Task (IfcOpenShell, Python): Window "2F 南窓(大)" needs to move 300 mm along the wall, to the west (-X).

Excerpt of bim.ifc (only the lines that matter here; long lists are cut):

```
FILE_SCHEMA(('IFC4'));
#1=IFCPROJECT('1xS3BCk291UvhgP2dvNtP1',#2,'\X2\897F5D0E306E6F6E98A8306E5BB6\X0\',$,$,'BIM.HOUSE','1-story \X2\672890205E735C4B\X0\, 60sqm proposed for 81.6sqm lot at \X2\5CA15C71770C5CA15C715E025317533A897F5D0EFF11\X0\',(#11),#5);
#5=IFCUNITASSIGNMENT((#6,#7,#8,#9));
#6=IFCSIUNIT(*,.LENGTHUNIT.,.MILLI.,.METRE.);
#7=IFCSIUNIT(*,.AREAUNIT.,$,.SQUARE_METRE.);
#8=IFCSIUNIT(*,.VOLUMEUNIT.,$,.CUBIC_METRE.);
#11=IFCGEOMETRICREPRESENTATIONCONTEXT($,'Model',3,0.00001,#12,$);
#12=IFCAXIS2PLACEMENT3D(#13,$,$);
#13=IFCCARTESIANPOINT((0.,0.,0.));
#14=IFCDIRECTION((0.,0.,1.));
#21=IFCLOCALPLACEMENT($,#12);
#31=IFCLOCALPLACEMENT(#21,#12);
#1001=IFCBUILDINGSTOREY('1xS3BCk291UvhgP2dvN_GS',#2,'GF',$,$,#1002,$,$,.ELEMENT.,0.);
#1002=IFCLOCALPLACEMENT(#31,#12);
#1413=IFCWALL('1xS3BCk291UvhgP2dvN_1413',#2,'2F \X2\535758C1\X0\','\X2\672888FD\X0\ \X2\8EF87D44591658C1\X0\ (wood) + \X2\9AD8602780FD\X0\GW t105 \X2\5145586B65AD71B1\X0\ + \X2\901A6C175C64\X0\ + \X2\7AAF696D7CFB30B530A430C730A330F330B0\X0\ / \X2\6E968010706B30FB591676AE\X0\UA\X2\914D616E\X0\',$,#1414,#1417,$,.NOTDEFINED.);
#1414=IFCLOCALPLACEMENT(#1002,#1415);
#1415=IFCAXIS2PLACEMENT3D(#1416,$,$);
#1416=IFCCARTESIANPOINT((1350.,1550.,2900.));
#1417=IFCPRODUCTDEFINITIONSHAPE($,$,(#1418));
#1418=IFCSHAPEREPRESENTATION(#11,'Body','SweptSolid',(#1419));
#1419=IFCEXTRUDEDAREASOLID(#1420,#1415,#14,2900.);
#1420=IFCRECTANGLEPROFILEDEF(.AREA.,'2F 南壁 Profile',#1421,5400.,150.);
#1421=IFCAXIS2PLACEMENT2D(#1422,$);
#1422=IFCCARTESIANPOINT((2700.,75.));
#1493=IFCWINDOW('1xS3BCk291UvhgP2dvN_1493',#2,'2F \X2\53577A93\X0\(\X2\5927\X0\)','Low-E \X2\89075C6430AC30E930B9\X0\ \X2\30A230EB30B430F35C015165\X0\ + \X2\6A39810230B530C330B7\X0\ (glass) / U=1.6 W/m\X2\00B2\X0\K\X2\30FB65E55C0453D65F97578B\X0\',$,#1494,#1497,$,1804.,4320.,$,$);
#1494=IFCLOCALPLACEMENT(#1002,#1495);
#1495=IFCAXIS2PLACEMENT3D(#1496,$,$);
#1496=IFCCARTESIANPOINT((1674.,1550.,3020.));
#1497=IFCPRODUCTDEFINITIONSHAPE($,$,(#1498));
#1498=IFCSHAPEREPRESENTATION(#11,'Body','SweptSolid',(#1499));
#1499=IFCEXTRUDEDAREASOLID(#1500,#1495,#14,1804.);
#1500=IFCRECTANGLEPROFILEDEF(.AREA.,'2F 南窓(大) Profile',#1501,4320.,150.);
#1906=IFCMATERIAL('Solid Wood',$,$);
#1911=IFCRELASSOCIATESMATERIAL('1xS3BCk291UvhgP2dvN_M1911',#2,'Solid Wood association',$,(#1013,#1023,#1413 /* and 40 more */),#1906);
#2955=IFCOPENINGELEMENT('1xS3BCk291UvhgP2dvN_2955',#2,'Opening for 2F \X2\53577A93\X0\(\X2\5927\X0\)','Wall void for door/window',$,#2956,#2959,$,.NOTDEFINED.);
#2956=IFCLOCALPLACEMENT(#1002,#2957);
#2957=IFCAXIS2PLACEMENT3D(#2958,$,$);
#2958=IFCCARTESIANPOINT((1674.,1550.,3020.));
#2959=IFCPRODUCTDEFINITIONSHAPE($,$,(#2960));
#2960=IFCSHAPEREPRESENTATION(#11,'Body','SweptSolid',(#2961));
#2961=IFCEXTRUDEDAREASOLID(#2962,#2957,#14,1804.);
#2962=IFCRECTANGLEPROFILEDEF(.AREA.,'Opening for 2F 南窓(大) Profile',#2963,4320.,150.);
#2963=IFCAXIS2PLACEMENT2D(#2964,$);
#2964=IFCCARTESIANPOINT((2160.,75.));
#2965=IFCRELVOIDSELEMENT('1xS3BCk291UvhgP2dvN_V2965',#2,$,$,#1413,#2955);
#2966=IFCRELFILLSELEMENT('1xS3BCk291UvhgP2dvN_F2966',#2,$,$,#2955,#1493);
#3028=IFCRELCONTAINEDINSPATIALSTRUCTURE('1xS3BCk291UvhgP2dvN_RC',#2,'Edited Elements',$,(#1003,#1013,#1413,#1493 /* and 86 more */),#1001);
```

```python
import ifcopenshell
import ifcopenshell.api.geometry
import ifcopenshell.util.placement
import ifcopenshell.util.unit

model = ifcopenshell.open("bim.ifc")
unit_scale = ifcopenshell.util.unit.calculate_unit_scale(model)

window = model.by_id(1493)
opening = window.FillsVoids[0].RelatingOpeningElement
wall = opening.VoidsElements[0].RelatingBuildingElement

wall_matrix = ifcopenshell.util.placement.get_local_placement(wall.ObjectPlacement)
shift = wall_matrix[:3, 0] * -0.3 / unit_scale
before = ifcopenshell.util.placement.get_local_placement(window.ObjectPlacement)[:3, 3].copy()

# The window is not placed relative to its opening, so move both.
for product in (opening, window):
    matrix = ifcopenshell.util.placement.get_local_placement(product.ObjectPlacement)
    matrix[:3, 3] += shift
    ifcopenshell.api.geometry.edit_object_placement(model, product=product, matrix=matrix, is_si=False)

after = ifcopenshell.util.placement.get_local_placement(window.ObjectPlacement)[:3, 3]
print("window moved by", (after - before).round(3) + 0.0)

model.write("bim_v2.ifc")
```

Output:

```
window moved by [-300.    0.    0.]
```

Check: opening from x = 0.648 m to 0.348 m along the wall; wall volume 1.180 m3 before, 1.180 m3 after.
